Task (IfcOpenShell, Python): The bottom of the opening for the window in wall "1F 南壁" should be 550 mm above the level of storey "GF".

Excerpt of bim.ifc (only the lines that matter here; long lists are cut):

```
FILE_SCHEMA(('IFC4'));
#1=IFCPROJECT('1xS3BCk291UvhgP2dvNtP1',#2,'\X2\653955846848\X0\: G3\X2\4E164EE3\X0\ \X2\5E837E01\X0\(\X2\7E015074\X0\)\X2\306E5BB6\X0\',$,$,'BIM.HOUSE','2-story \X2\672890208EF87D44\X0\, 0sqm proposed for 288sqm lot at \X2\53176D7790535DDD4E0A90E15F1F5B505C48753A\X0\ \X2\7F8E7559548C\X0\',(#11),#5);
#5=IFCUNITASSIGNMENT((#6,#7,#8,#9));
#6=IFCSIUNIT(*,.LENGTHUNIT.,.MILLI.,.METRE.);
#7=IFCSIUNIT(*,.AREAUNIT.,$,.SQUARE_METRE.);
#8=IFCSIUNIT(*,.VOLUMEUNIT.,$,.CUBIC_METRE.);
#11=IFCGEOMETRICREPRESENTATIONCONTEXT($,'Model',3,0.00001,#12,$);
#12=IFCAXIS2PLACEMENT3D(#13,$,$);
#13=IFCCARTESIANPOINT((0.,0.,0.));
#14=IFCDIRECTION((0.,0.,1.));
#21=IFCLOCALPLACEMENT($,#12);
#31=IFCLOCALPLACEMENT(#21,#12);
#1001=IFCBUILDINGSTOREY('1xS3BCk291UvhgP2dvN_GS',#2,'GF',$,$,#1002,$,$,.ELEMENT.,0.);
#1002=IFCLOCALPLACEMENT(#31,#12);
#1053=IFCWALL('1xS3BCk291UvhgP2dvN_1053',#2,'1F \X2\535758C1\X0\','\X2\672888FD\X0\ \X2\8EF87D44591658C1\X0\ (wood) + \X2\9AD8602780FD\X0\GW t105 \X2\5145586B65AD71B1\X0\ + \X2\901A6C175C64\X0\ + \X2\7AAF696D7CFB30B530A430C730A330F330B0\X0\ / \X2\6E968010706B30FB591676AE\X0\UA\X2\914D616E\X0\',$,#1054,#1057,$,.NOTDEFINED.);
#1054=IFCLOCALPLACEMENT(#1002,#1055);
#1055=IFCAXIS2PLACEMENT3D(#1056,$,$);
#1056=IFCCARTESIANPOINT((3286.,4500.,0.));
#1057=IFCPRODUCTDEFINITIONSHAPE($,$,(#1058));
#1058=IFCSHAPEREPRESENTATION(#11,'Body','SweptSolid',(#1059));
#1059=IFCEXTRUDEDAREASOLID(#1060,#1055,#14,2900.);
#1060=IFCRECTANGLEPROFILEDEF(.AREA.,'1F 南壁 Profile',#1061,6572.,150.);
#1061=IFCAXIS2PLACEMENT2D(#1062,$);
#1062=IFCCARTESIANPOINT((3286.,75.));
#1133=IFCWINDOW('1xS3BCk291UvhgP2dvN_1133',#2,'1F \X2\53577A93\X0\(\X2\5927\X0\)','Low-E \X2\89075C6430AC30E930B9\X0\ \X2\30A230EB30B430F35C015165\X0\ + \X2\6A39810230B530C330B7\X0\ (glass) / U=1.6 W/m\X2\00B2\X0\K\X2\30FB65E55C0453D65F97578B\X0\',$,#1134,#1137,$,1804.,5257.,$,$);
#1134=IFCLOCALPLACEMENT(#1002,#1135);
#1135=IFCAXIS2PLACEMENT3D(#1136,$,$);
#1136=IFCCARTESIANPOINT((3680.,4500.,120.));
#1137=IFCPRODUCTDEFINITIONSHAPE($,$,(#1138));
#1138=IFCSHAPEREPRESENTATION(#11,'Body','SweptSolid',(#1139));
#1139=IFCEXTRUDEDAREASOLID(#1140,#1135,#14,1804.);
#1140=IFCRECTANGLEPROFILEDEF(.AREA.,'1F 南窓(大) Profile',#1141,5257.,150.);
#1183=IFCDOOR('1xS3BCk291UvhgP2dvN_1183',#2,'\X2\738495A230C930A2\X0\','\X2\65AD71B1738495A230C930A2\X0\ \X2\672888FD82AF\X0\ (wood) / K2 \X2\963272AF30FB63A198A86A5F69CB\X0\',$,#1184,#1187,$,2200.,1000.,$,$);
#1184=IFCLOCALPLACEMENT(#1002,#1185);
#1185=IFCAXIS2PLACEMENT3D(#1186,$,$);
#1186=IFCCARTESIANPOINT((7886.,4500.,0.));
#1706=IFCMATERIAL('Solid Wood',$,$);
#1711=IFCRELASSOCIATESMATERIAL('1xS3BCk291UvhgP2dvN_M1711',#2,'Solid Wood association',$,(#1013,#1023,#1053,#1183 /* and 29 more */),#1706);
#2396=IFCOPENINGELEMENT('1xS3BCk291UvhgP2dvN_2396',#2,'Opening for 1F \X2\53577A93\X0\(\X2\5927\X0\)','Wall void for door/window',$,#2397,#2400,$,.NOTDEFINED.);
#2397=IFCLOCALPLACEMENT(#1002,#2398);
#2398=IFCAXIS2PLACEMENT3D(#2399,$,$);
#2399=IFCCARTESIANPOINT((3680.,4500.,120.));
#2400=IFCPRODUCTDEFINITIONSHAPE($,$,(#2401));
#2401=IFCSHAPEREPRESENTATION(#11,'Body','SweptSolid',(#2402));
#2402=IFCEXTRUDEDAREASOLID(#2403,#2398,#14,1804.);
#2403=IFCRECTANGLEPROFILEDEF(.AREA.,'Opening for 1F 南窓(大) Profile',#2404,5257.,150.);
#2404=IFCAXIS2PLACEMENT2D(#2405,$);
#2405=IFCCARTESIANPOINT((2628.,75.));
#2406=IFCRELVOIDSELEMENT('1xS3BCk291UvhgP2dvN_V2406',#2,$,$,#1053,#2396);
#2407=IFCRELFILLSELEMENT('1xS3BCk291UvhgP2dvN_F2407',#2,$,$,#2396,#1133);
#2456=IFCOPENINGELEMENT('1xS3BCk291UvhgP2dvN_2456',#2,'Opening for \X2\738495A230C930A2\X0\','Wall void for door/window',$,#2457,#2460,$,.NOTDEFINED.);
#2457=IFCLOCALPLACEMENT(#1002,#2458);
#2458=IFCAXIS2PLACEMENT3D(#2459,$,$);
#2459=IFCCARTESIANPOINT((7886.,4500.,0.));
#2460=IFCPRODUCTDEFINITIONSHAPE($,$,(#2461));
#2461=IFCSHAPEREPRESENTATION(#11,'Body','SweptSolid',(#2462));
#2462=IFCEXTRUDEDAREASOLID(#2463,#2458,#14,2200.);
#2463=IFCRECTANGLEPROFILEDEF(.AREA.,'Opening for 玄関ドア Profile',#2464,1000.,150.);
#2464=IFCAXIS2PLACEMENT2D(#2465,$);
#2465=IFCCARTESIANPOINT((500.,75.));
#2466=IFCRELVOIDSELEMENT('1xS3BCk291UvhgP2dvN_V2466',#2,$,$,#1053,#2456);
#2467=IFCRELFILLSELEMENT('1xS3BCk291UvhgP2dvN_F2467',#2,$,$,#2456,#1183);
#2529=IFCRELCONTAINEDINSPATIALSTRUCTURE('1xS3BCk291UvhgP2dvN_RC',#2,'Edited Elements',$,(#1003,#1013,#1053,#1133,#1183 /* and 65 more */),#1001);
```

```python
import numpy as np
import ifcopenshell
import ifcopenshell.api.geometry
import ifcopenshell.geom
import ifcopenshell.util.element
import ifcopenshell.util.placement
import ifcopenshell.util.shape
import ifcopenshell.util.unit

model = ifcopenshell.open("bim.ifc")
unit_scale = ifcopenshell.util.unit.calculate_unit_scale(model)

window = model.by_guid("1xS3BCk291UvhgP2dvN_1133")
opening = window.FillsVoids[0].RelatingOpeningElement
storey = ifcopenshell.util.element.get_container(window, ifc_class="IfcBuildingStorey")
level = ifcopenshell.util.placement.get_local_placement(storey.ObjectPlacement)[2, 3]

# The opening's origin need not be at the sill, so measure its lowest point.
shape = ifcopenshell.geom.create_shape(ifcopenshell.geom.settings(), opening)
bottom = ifcopenshell.util.shape.get_shape_bottom_elevation(shape, shape.geometry) / unit_scale
dz = level + 550.0 - bottom

shift = np.array([0.0, 0.0, dz])
# The window is not placed relative to its opening, so move both.
for product in (opening, window):
    matrix = ifcopenshell.util.placement.get_local_placement(product.ObjectPlacement)
    matrix[:3, 3] += shift
    ifcopenshell.api.geometry.edit_object_placement(model, product=product, matrix=matrix, is_si=False)

print(f"moved by {dz * unit_scale:+.3f} m")

model.write("bim_updated.ifc")
```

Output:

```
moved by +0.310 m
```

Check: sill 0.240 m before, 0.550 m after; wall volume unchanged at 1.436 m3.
